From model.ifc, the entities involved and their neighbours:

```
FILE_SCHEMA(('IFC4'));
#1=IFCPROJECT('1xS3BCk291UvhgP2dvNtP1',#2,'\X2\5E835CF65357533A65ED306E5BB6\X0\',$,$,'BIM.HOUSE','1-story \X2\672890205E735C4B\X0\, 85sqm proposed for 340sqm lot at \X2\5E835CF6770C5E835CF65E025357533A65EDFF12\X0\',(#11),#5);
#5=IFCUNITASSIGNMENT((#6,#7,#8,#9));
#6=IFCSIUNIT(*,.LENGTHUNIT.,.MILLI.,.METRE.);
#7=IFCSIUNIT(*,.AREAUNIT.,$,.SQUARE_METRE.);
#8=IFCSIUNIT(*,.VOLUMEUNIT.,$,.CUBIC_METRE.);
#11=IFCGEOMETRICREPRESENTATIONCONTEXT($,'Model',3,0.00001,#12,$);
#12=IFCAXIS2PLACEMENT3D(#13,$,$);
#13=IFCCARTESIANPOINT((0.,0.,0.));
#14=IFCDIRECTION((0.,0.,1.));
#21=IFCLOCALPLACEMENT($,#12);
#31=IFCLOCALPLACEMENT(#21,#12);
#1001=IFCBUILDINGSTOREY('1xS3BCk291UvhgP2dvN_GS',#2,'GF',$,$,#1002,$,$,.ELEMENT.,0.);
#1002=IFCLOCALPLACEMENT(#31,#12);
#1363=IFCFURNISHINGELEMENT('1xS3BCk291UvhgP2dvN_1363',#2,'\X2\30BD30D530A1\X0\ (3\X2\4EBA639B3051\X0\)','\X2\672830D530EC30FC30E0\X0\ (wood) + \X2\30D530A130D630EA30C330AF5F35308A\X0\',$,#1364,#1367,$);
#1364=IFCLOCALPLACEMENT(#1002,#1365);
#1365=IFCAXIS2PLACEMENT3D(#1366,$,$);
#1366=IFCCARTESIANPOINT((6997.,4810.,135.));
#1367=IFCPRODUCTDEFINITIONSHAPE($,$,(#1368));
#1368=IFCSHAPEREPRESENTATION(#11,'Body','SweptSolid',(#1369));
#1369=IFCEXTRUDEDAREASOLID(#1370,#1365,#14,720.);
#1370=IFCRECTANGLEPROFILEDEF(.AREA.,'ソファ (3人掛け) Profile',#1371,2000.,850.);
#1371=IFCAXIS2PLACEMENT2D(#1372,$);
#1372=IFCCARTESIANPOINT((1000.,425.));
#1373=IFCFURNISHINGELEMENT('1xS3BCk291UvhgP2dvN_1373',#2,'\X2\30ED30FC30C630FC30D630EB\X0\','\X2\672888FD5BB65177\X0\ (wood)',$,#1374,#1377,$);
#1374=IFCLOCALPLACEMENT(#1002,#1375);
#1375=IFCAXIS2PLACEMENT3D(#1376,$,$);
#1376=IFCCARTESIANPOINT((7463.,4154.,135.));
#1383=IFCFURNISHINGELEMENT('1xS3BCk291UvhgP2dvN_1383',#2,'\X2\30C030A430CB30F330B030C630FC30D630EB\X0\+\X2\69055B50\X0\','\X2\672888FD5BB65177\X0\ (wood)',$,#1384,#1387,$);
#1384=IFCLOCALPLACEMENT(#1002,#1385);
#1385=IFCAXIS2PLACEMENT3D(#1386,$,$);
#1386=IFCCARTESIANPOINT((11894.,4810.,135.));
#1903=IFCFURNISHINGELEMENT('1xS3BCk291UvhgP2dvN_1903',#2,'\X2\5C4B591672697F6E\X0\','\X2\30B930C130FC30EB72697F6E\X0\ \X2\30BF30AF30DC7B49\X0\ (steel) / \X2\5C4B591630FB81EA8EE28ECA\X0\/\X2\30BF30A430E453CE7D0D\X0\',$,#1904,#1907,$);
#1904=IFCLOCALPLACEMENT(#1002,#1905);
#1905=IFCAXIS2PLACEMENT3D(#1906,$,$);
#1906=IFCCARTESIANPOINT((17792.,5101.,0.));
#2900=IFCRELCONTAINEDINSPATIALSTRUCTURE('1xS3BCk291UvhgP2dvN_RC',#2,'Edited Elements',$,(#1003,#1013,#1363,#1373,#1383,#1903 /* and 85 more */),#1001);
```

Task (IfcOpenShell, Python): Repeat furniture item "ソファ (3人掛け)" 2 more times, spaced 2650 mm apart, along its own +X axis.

```python
import ifcopenshell
import ifcopenshell.api.geometry
import ifcopenshell.api.root
import ifcopenshell.util.element
import ifcopenshell.util.placement

model = ifcopenshell.open("model.ifc")


def reuse_history(source, copy):
    """copy_class also copies each property set's owner history, people and application; keep the originals."""
    for rel in copy.IsDefinedBy:
        if rel.is_a("IfcRelDefinesByProperties") and (history := rel.RelatingPropertyDefinition.OwnerHistory):
            rel.RelatingPropertyDefinition.OwnerHistory = source.OwnerHistory
            ifcopenshell.util.element.remove_deep2(model, history)


source = model.by_guid("1xS3BCk291UvhgP2dvN_1363")
base = ifcopenshell.util.placement.get_local_placement(source.ObjectPlacement)
step = base[:3, 0] * 2650.0

for i in range(1, 3):
    copy = ifcopenshell.api.root.copy_class(model, product=source)
    copy.Representation = ifcopenshell.util.element.copy_deep(
        model, source.Representation, exclude=["IfcGeometricRepresentationContext", "IfcRepresentationMap"]
    )
    reuse_history(source, copy)
    matrix = base.copy()
    matrix[:3, 3] += i * step
    print("added at", matrix[:3, 3].round(3) + 0.0)
    ifcopenshell.api.geometry.edit_object_placement(model, product=copy, matrix=matrix, is_si=False)

model.write("model_v2.ifc")
```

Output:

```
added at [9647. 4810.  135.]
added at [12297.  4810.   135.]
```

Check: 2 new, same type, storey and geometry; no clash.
